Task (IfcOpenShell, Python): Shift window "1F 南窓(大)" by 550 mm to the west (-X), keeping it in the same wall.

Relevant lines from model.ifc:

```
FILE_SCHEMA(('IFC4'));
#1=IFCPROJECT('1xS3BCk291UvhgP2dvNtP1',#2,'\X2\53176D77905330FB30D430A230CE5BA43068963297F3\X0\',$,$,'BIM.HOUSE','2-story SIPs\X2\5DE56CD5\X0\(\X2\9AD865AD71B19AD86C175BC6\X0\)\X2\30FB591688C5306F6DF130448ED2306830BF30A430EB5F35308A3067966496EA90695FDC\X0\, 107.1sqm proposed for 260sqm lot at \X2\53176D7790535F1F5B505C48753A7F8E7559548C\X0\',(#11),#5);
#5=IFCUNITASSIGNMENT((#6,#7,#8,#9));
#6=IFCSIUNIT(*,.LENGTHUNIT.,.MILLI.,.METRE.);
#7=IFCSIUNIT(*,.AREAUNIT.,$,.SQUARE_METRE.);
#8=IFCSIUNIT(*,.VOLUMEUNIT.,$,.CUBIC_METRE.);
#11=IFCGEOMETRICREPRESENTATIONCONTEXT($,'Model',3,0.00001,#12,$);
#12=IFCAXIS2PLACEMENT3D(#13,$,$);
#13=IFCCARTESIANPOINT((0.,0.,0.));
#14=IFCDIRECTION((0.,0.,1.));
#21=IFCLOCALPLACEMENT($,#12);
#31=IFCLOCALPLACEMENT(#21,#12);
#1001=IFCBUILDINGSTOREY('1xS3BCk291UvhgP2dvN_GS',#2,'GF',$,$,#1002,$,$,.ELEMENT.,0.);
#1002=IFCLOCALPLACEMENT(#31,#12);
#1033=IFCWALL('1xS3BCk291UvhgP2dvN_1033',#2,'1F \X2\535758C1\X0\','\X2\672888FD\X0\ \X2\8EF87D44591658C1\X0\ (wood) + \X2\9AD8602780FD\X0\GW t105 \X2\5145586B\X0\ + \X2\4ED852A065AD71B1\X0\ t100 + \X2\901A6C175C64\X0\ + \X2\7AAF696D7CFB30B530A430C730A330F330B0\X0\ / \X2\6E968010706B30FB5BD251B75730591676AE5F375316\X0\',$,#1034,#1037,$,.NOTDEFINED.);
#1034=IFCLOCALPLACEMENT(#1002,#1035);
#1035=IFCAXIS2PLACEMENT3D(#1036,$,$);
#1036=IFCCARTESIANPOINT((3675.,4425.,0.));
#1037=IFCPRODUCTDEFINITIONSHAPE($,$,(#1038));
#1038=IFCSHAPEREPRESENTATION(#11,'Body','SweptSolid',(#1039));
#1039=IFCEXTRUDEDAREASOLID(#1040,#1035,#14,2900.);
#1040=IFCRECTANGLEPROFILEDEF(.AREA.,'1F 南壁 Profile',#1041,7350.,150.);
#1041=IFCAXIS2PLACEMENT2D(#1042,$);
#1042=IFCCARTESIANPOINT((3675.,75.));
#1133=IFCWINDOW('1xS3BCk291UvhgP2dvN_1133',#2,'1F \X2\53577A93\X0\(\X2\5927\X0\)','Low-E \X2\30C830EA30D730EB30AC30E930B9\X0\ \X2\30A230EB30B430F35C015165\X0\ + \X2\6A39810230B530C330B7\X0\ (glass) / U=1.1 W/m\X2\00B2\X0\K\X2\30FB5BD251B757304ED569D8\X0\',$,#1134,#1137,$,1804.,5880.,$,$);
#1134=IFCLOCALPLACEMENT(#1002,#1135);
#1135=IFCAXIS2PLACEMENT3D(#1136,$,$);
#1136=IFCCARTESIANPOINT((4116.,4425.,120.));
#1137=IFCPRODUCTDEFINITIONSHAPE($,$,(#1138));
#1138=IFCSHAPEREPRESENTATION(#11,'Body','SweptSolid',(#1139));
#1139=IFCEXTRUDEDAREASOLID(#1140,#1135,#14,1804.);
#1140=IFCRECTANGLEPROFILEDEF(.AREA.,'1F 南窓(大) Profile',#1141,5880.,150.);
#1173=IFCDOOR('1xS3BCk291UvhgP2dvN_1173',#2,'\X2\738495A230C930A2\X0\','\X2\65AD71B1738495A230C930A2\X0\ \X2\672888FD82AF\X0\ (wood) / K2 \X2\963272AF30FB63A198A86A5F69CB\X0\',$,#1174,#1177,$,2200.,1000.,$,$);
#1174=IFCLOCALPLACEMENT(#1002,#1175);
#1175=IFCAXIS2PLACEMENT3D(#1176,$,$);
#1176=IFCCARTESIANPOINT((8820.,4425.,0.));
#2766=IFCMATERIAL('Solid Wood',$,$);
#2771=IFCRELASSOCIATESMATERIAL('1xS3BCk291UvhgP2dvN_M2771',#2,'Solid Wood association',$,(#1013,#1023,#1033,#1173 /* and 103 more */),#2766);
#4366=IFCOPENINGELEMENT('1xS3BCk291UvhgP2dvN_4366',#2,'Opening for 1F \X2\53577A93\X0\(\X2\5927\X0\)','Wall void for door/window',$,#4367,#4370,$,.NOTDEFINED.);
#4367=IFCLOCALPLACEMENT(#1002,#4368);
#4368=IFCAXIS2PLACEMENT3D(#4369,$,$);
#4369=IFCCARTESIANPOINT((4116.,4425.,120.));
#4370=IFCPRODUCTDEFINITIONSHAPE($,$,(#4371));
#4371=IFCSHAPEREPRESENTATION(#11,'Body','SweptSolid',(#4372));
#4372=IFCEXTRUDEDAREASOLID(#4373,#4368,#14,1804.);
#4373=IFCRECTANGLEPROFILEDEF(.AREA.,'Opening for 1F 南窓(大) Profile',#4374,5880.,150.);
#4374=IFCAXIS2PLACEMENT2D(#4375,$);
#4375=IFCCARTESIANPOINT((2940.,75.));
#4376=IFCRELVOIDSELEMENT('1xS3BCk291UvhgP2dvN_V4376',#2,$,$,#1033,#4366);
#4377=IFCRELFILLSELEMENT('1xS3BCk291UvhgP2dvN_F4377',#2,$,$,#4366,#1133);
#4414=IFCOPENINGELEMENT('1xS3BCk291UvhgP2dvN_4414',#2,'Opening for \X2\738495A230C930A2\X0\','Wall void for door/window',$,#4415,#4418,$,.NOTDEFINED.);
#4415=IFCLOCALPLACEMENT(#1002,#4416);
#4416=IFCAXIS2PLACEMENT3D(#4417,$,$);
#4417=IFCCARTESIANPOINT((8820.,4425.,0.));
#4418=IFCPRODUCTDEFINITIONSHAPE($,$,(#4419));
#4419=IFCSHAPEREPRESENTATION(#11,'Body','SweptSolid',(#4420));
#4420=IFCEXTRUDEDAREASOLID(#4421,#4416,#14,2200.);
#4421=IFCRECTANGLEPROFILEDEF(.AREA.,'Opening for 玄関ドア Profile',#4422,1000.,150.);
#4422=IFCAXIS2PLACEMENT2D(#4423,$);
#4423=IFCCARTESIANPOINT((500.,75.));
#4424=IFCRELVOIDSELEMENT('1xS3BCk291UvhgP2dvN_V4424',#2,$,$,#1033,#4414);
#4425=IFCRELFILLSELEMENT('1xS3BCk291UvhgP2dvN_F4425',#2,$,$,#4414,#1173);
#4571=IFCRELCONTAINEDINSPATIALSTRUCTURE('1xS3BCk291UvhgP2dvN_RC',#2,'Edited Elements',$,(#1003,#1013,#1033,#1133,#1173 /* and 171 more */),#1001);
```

```python
import ifcopenshell
import ifcopenshell.api.geometry
import ifcopenshell.util.placement
import ifcopenshell.util.unit

model = ifcopenshell.open("model.ifc")
unit_scale = ifcopenshell.util.unit.calculate_unit_scale(model)

window = model.by_guid("1xS3BCk291UvhgP2dvN_1133")
opening = window.FillsVoids[0].RelatingOpeningElement
wall = opening.VoidsElements[0].RelatingBuildingElement

wall_matrix = ifcopenshell.util.placement.get_local_placement(wall.ObjectPlacement)
shift = wall_matrix[:3, 0] * -0.55 / unit_scale
before = ifcopenshell.util.placement.get_local_placement(window.ObjectPlacement)[:3, 3].copy()

# The window is not placed relative to its opening, so move both.
for product in (opening, window):
    matrix = ifcopenshell.util.placement.get_local_placement(product.ObjectPlacement)
    matrix[:3, 3] += shift
    ifcopenshell.api.geometry.edit_object_placement(model, product=product, matrix=matrix, is_si=False)

after = ifcopenshell.util.placement.get_local_placement(window.ObjectPlacement)[:3, 3]
print("window moved by", (after - before).round(3) + 0.0)

model.write("model_edited.ifc")
```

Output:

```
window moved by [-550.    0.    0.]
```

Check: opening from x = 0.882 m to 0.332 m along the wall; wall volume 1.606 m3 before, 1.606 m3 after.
